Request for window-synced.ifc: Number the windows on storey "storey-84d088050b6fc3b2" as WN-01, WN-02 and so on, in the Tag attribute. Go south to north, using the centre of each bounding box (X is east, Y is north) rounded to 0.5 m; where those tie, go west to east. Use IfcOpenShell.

First a look at what the model holds.

```python
import ifcopenshell
import ifcopenshell.util.element
import ifcopenshell.util.placement

model = ifcopenshell.open("window-synced.ifc")
print(model.schema)
storey = next(s for s in model.by_type("IfcBuildingStorey") if s.Name == "storey-84d088050b6fc3b2")
windows = [e for e in ifcopenshell.util.element.get_decomposition(storey) if e.is_a("IfcWindow")]
for e in sorted(windows, key=lambda e: e.id()):
    origin = ifcopenshell.util.placement.get_local_placement(e.ObjectPlacement)[:3, 3]
    print(e.id(), e.Tag, e.Name, origin.round(2) + 0.0, sep=" | ")
```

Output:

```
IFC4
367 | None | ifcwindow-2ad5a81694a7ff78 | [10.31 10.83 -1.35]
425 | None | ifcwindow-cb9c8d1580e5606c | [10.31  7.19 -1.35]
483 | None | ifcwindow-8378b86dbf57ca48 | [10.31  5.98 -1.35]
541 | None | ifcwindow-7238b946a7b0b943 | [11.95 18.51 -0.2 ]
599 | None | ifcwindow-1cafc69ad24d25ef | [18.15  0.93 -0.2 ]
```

```python
import ifcopenshell
import ifcopenshell.geom
import ifcopenshell.util.element
import ifcopenshell.util.shape

model = ifcopenshell.open("window-synced.ifc")
settings = ifcopenshell.geom.settings()
settings.set("use-world-coords", True)


def centre(element):
    shape = ifcopenshell.geom.create_shape(settings, element)
    return ifcopenshell.util.shape.get_bbox_centroid(shape.geometry)


storey = next(s for s in model.by_type("IfcBuildingStorey") if s.Name == "storey-84d088050b6fc3b2")
windows = [e for e in ifcopenshell.util.element.get_decomposition(storey) if e.is_a("IfcWindow")]

# Insertion points can sit at a corner or the storey origin, so sort by the geometry (in metres).
centres = {e: centre(e) for e in windows}
windows.sort(key=lambda e: (round(centres[e][1] / 0.5), centres[e][0]))

for i, e in enumerate(windows, start=1):
    number = f"WN-{i:02d}"
    e.Tag = number
    print(e.id(), number)

model.write("window-synced_edited.ifc")
```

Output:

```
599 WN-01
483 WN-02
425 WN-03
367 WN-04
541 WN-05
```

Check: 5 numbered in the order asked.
